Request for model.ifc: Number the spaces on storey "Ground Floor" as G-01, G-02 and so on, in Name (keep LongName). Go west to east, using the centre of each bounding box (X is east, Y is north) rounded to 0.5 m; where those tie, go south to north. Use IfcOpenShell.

First a look at what the model holds.

```python
import ifcopenshell
import ifcopenshell.util.element
import ifcopenshell.util.placement

model = ifcopenshell.open("model.ifc")
print(model.schema)
storey = next(s for s in model.by_type("IfcBuildingStorey") if s.Name == "Ground Floor")
spaces = [e for e in ifcopenshell.util.element.get_decomposition(storey) if e.is_a("IfcSpace")]
for e in sorted(spaces, key=lambda e: e.id()):
    origin = ifcopenshell.util.placement.get_local_placement(e.ObjectPlacement)[:3, 3]
    print(e.id(), e.Name, e.LongName, origin.round(2) + 0.0, sep=" | ")
```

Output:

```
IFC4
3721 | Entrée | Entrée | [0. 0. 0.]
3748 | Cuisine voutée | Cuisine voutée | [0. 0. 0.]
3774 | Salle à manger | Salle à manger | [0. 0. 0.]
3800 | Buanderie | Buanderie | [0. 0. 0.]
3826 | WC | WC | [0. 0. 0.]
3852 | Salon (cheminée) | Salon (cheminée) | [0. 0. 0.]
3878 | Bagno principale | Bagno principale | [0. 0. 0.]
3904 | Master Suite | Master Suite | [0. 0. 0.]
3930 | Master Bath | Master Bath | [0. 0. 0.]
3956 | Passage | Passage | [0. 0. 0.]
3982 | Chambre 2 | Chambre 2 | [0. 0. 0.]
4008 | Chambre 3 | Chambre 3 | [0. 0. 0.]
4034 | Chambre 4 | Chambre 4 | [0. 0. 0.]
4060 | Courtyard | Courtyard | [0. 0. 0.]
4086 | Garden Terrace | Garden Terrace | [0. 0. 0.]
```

```python
import ifcopenshell
import ifcopenshell.geom
import ifcopenshell.util.element
import ifcopenshell.util.shape

model = ifcopenshell.open("model.ifc")
settings = ifcopenshell.geom.settings()
settings.set("use-world-coords", True)


def centre(element):
    shape = ifcopenshell.geom.create_shape(settings, element)
    return ifcopenshell.util.shape.get_bbox_centroid(shape.geometry)


storey = next(s for s in model.by_type("IfcBuildingStorey") if s.Name == "Ground Floor")
spaces = [e for e in ifcopenshell.util.element.get_decomposition(storey) if e.is_a("IfcSpace")]

# Insertion points can sit at a corner or the storey origin, so sort by the geometry (in metres).
centres = {e: centre(e) for e in spaces}
spaces.sort(key=lambda e: (round(centres[e][0] / 0.5), centres[e][1]))

for i, e in enumerate(spaces, start=1):
    number = f"G-{i:02d}"
    e.Name = number
    print(e.id(), number)

model.write("model_edited.ifc")
```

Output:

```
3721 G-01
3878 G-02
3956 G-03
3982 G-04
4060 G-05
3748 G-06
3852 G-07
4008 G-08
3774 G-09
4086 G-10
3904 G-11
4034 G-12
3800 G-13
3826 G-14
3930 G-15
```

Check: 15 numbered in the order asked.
